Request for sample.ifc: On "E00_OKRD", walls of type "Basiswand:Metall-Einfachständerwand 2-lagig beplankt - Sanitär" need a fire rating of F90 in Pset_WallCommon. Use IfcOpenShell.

First a look at what the model holds.

```python
import ifcopenshell
import ifcopenshell.util.element

model = ifcopenshell.open("sample.ifc")
print(model.schema)
storey = next(s for s in model.by_type("IfcBuildingStorey") if s.Name == "E00_OKRD")
walls = [e for e in ifcopenshell.util.element.get_decomposition(storey) if e.is_a("IfcWall")]
seen = {}
for e in walls:
    element_type = ifcopenshell.util.element.get_type(e)
    key = (element_type.Name if element_type != e and element_type else None, ifcopenshell.util.element.get_pset(e, "Pset_WallCommon", "FireRating"))
    seen[key] = seen.get(key, 0) + 1
for (name, value), count in sorted(seen.items(), key=str):
    print(count, "x", name, "|", value)
```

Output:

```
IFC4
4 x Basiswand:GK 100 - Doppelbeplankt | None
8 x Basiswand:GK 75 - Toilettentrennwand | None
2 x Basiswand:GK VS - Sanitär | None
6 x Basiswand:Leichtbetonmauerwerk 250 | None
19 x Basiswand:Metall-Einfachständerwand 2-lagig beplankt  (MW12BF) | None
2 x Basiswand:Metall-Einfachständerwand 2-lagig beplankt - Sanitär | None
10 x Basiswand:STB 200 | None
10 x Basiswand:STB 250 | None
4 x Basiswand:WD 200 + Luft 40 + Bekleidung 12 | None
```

```python
import ifcopenshell
import ifcopenshell.api.pset
import ifcopenshell.util.element

model = ifcopenshell.open("sample.ifc")

storey = next(s for s in model.by_type("IfcBuildingStorey") if s.Name == "E00_OKRD")
walls = [e for e in ifcopenshell.util.element.get_decomposition(storey) if e.is_a("IfcWall")]

count = 0
for e in walls:
    element_type = ifcopenshell.util.element.get_type(e)
    if element_type in (None, e) or element_type.Name != "Basiswand:Metall-Einfachständerwand 2-lagig beplankt - Sanitär":
        continue
    # add_pset returns the element's existing set when there is one.
    pset = ifcopenshell.api.pset.add_pset(model, product=e, name="Pset_WallCommon")
    ifcopenshell.api.pset.edit_pset(model, pset=pset, properties={"FireRating": "F90"})
    count += 1

print(count, "walls updated")

model.write("sample_rev.ifc")
```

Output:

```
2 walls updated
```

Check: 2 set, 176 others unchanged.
